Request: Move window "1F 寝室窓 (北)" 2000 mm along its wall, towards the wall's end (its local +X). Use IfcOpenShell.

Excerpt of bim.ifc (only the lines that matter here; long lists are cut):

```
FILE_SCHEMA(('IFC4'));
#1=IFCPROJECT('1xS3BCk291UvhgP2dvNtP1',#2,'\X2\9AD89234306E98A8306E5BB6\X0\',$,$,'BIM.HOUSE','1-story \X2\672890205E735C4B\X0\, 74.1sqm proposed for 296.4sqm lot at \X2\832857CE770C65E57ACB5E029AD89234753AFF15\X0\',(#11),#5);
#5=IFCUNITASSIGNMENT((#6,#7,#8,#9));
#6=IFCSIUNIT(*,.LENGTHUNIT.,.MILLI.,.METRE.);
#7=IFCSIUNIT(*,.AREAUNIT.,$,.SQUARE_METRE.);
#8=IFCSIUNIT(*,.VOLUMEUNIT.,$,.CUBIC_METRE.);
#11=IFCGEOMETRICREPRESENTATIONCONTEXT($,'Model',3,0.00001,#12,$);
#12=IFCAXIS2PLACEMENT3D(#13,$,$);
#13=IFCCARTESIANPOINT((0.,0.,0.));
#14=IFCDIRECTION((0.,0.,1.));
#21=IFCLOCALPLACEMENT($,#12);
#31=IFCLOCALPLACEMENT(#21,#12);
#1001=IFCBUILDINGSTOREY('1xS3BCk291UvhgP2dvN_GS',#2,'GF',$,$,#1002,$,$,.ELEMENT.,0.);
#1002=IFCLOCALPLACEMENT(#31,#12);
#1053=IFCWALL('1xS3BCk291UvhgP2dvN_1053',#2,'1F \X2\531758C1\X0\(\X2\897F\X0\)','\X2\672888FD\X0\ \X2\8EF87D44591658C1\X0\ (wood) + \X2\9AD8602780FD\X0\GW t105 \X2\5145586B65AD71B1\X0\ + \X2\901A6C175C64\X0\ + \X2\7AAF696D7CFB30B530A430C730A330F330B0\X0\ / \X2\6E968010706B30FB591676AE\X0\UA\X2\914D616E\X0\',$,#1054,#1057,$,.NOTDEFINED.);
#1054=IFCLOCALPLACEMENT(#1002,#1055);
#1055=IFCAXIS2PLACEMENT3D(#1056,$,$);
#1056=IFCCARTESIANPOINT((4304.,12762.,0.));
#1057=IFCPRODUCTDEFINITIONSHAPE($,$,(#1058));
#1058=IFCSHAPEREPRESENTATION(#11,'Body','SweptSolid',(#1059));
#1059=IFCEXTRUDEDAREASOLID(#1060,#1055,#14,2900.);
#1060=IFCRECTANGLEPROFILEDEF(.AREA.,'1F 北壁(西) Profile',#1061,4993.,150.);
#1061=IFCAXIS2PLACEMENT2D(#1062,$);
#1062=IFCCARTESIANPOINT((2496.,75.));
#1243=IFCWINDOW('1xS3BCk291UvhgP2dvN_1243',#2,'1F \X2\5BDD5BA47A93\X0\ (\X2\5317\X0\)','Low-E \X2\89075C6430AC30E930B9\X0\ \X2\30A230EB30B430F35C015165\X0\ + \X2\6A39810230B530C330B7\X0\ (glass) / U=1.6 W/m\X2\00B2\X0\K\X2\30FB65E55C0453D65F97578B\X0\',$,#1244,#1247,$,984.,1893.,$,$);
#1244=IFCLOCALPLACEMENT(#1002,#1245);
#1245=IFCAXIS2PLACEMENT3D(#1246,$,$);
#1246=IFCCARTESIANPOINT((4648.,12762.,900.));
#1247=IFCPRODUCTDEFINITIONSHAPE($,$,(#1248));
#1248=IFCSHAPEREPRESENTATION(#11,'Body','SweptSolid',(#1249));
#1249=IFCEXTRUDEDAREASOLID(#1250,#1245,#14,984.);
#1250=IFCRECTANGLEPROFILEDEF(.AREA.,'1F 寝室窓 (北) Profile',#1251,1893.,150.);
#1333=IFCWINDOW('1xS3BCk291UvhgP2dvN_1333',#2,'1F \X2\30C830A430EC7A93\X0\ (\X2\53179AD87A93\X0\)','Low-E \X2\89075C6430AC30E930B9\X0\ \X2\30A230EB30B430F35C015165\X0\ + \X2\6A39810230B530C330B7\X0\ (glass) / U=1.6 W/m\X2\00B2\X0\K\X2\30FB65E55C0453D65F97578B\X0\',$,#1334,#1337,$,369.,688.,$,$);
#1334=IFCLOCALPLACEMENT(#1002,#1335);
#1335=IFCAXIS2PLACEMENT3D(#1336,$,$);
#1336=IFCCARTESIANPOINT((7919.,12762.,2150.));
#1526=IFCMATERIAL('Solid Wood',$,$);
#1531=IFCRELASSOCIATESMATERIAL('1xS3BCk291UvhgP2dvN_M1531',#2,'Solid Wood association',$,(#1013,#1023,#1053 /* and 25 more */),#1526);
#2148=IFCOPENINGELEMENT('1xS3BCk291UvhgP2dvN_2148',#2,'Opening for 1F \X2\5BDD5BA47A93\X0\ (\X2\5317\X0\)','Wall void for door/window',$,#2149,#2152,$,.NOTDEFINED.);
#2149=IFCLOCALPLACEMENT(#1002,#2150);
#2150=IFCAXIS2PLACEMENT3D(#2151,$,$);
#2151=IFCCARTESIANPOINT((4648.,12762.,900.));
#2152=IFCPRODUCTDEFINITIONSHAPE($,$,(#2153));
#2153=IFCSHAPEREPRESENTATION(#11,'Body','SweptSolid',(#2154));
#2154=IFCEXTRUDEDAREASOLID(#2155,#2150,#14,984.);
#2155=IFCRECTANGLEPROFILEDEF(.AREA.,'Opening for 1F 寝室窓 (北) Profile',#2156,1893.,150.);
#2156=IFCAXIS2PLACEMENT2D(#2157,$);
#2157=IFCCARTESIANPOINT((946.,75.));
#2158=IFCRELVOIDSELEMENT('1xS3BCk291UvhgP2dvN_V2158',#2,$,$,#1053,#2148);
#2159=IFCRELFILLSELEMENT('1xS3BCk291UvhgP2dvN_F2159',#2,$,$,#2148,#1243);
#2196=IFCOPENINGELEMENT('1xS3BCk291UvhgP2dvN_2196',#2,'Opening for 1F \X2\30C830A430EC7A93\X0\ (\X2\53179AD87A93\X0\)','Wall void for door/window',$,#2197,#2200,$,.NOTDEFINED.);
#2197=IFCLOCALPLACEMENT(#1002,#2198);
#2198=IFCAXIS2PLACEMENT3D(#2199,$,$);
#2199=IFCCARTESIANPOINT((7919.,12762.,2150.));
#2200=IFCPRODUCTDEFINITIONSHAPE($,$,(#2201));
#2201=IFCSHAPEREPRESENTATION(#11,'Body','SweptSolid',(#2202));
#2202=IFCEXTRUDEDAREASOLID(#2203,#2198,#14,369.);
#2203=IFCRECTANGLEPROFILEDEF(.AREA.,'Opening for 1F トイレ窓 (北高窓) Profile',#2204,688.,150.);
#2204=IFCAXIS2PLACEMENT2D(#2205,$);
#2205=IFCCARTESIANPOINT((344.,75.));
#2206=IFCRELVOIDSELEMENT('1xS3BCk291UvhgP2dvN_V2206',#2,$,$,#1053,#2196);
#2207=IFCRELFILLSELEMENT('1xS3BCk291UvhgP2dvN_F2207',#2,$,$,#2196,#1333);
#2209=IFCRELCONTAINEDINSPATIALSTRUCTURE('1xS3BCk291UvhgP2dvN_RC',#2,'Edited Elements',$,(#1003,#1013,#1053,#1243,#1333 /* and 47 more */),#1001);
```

```python
import ifcopenshell
import ifcopenshell.api.geometry
import ifcopenshell.util.placement
import ifcopenshell.util.unit

model = ifcopenshell.open("bim.ifc")
unit_scale = ifcopenshell.util.unit.calculate_unit_scale(model)

window = model.by_id(1243)
opening = window.FillsVoids[0].RelatingOpeningElement
wall = opening.VoidsElements[0].RelatingBuildingElement

wall_matrix = ifcopenshell.util.placement.get_local_placement(wall.ObjectPlacement)
shift = wall_matrix[:3, 0] * 2 / unit_scale
before = ifcopenshell.util.placement.get_local_placement(window.ObjectPlacement)[:3, 3].copy()

# The window is not placed relative to its opening, so move both.
for product in (opening, window):
    matrix = ifcopenshell.util.placement.get_local_placement(product.ObjectPlacement)
    matrix[:3, 3] += shift
    ifcopenshell.api.geometry.edit_object_placement(model, product=product, matrix=matrix, is_si=False)

after = ifcopenshell.util.placement.get_local_placement(window.ObjectPlacement)[:3, 3]
print("window moved by", (after - before).round(3) + 0.0)

model.write("bim_edited.ifc")
```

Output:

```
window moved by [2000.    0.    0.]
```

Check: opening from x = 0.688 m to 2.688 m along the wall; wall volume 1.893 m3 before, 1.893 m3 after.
